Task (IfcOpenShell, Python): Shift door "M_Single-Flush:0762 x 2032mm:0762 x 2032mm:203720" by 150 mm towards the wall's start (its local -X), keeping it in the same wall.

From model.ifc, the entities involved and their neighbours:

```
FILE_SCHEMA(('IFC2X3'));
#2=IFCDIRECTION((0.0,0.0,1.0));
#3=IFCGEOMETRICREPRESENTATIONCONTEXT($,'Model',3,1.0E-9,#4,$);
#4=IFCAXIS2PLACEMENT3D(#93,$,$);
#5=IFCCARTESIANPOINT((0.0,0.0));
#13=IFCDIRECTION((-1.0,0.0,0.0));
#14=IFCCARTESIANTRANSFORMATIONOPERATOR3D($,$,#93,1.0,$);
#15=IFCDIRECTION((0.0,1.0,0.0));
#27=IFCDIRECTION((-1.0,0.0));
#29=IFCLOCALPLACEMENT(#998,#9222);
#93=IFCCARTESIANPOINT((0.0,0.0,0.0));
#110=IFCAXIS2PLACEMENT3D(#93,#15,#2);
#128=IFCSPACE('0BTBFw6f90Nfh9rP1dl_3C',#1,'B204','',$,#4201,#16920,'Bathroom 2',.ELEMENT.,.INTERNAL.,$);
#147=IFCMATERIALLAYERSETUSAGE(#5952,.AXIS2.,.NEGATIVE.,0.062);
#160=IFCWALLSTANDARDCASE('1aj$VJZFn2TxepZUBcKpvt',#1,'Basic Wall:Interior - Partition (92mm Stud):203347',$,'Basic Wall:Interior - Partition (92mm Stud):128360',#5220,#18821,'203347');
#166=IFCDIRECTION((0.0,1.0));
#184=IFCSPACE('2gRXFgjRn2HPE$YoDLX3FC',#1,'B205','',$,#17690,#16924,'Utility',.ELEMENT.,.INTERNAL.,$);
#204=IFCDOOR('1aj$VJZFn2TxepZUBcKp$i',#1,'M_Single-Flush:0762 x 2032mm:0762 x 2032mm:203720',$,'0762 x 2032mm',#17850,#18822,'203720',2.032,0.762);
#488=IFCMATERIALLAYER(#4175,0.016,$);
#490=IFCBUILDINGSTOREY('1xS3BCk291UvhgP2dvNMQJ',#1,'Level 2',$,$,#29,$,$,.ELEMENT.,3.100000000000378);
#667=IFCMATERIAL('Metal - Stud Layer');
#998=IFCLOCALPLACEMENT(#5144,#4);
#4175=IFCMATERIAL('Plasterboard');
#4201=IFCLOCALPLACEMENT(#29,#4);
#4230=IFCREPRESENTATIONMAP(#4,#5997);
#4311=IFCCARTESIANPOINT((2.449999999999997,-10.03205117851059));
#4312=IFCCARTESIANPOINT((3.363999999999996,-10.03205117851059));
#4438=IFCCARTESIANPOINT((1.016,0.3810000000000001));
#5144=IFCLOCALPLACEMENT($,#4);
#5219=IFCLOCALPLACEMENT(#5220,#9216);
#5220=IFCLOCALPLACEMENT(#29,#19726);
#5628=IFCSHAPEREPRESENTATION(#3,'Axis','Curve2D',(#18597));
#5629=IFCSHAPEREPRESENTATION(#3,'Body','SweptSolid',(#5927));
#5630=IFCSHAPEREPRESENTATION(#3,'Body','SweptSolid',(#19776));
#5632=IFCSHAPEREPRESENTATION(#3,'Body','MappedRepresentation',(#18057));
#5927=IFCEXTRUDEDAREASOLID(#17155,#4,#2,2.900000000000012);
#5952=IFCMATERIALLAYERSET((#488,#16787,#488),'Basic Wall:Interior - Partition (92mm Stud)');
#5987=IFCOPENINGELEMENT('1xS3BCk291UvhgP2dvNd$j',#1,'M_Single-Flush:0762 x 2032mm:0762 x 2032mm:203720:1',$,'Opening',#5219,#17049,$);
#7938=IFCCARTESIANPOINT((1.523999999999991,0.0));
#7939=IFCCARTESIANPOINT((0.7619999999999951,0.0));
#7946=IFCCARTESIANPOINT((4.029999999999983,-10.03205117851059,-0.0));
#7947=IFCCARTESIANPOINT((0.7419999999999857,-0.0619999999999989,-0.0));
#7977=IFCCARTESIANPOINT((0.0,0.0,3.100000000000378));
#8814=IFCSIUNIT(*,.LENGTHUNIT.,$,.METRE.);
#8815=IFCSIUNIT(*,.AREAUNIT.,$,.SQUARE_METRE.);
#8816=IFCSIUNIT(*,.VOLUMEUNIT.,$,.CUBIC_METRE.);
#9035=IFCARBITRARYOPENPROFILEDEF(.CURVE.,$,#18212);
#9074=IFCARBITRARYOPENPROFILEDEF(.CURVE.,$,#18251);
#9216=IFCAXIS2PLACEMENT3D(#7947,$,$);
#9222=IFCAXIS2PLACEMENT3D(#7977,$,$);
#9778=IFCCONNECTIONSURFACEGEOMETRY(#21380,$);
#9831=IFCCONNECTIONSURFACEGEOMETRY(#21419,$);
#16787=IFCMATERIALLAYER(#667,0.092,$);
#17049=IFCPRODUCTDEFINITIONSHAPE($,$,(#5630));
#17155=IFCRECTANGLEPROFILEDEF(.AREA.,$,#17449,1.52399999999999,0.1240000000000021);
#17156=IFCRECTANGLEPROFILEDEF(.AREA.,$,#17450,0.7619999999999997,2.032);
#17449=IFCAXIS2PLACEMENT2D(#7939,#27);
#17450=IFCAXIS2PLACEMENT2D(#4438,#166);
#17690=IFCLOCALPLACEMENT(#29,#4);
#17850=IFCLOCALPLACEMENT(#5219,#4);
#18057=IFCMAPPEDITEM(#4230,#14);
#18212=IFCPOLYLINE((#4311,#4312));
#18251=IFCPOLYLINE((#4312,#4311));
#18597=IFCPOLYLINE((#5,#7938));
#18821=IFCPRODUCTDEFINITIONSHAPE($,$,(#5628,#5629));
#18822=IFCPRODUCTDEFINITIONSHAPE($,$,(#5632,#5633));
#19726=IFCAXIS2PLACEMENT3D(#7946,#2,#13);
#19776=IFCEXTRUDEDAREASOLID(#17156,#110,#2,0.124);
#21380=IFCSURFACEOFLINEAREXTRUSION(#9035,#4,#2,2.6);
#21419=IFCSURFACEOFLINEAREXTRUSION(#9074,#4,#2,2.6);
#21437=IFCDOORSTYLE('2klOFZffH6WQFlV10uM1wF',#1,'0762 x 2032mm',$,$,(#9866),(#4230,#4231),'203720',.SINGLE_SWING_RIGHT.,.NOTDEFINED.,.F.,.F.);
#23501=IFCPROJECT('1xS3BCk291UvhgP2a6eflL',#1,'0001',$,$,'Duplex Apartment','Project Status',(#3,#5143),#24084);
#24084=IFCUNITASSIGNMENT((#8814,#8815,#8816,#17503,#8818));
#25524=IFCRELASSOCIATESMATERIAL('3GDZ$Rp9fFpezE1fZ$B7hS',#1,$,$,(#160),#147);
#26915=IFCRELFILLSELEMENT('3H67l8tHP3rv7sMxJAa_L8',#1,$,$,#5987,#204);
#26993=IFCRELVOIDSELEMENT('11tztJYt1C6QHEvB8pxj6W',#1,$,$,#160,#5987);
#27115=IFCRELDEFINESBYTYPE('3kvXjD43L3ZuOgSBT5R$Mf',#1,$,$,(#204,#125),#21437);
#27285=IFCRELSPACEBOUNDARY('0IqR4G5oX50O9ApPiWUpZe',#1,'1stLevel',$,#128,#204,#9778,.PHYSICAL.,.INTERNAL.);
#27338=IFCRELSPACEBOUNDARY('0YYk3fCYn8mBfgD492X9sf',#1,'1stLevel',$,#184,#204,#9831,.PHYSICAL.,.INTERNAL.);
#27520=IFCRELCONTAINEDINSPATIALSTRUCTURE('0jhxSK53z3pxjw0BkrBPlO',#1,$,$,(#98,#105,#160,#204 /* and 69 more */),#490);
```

```python
import numpy as np
import ifcopenshell
import ifcopenshell.api.geometry
import ifcopenshell.util.placement
import ifcopenshell.util.unit

model = ifcopenshell.open("model.ifc")
unit_scale = ifcopenshell.util.unit.calculate_unit_scale(model)

door = model.by_guid("1aj$VJZFn2TxepZUBcKp$i")
opening = door.FillsVoids[0].RelatingOpeningElement
wall = opening.VoidsElements[0].RelatingBuildingElement

wall_matrix = ifcopenshell.util.placement.get_local_placement(wall.ObjectPlacement)
shift = wall_matrix[:3, 0] * -0.15 / unit_scale
before = ifcopenshell.util.placement.get_local_placement(door.ObjectPlacement)[:3, 3].copy()

# The door is placed relative to its opening, so it follows when the opening moves.
matrix = ifcopenshell.util.placement.get_local_placement(opening.ObjectPlacement)
matrix[:3, 3] += shift
ifcopenshell.api.geometry.edit_object_placement(
    model, product=opening, matrix=matrix, is_si=False, should_transform_children=True
)

# Space boundary surfaces are stored in each space's coordinates; move them too.
for rel in door.ProvidesBoundaries:
    if not rel.ConnectionGeometry:
        continue
    surface = rel.ConnectionGeometry.SurfaceOnRelatingElement
    space_matrix = ifcopenshell.util.placement.get_local_placement(rel.RelatingSpace.ObjectPlacement)
    point = np.array(surface.Position.Location.Coordinates) + space_matrix[:3, :3].T @ shift
    surface.Position = model.createIfcAxis2Placement3D(
        model.createIfcCartesianPoint(point.tolist()), surface.Position.Axis, surface.Position.RefDirection
    )

after = ifcopenshell.util.placement.get_local_placement(door.ObjectPlacement)[:3, 3]
print("door moved by", (after - before).round(3) + 0.0)

model.write("model_updated.ifc")
```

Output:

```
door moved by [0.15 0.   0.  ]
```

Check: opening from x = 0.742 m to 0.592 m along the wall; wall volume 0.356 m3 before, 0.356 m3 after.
